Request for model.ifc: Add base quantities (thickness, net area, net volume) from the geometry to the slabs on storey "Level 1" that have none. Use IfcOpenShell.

First a look at what the model holds.

```python
import ifcopenshell
import ifcopenshell.util.element
import ifcopenshell.util.unit

model = ifcopenshell.open("model.ifc")
print(model.schema)
for unit_type in ("LENGTHUNIT", "AREAUNIT", "VOLUMEUNIT"):
    print(unit_type, ifcopenshell.util.unit.calculate_unit_scale(model, unit_type))
storey = next(s for s in model.by_type("IfcBuildingStorey") if s.Name == "Level 1")
slabs = [e for e in ifcopenshell.util.element.get_decomposition(storey) if e.is_a("IfcSlab")]
for e in sorted(slabs, key=lambda e: e.id()):
    print(e.id(), e.is_a(), e.Name, list(ifcopenshell.util.element.get_psets(e, qtos_only=True)), sep=" | ")
```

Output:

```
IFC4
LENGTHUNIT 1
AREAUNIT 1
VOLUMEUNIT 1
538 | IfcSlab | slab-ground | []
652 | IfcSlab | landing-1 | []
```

```python
import ifcopenshell
import ifcopenshell.api.pset
import ifcopenshell.geom
import ifcopenshell.util.element
import ifcopenshell.util.shape
import ifcopenshell.util.unit

model = ifcopenshell.open("model.ifc")
unit_scale = ifcopenshell.util.unit.calculate_unit_scale(model)
area_scale = ifcopenshell.util.unit.calculate_unit_scale(model, "AREAUNIT")
volume_scale = ifcopenshell.util.unit.calculate_unit_scale(model, "VOLUMEUNIT")
settings = ifcopenshell.geom.settings()

storey = next(s for s in model.by_type("IfcBuildingStorey") if s.Name == "Level 1")
slabs = [e for e in ifcopenshell.util.element.get_decomposition(storey) if e.is_a("IfcSlab")]

for e in sorted(slabs, key=lambda e: e.id()):
    if ifcopenshell.util.element.get_psets(e, qtos_only=True, should_inherit=False):
        continue
    # Geometry comes back in metres, in the element's own axes.
    shape = ifcopenshell.geom.create_shape(settings, e)
    values = {
        "Width": ifcopenshell.util.shape.get_z(shape.geometry) / unit_scale,
        "NetArea": ifcopenshell.util.shape.get_footprint_area(shape.geometry) / area_scale,
        "NetVolume": ifcopenshell.util.shape.get_volume(shape.geometry) / volume_scale,
    }
    qto = ifcopenshell.api.pset.add_qto(model, product=e, name="Qto_SlabBaseQuantities")
    ifcopenshell.api.pset.edit_qto(model, qto=qto, properties=values)
    print(e.id(), {k: round(v, 3) for k, v in values.items()})

model.write("model_rev.ifc")
```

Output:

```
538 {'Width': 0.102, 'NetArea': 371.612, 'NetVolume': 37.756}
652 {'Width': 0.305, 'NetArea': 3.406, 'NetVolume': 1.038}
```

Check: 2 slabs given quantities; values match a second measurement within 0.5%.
